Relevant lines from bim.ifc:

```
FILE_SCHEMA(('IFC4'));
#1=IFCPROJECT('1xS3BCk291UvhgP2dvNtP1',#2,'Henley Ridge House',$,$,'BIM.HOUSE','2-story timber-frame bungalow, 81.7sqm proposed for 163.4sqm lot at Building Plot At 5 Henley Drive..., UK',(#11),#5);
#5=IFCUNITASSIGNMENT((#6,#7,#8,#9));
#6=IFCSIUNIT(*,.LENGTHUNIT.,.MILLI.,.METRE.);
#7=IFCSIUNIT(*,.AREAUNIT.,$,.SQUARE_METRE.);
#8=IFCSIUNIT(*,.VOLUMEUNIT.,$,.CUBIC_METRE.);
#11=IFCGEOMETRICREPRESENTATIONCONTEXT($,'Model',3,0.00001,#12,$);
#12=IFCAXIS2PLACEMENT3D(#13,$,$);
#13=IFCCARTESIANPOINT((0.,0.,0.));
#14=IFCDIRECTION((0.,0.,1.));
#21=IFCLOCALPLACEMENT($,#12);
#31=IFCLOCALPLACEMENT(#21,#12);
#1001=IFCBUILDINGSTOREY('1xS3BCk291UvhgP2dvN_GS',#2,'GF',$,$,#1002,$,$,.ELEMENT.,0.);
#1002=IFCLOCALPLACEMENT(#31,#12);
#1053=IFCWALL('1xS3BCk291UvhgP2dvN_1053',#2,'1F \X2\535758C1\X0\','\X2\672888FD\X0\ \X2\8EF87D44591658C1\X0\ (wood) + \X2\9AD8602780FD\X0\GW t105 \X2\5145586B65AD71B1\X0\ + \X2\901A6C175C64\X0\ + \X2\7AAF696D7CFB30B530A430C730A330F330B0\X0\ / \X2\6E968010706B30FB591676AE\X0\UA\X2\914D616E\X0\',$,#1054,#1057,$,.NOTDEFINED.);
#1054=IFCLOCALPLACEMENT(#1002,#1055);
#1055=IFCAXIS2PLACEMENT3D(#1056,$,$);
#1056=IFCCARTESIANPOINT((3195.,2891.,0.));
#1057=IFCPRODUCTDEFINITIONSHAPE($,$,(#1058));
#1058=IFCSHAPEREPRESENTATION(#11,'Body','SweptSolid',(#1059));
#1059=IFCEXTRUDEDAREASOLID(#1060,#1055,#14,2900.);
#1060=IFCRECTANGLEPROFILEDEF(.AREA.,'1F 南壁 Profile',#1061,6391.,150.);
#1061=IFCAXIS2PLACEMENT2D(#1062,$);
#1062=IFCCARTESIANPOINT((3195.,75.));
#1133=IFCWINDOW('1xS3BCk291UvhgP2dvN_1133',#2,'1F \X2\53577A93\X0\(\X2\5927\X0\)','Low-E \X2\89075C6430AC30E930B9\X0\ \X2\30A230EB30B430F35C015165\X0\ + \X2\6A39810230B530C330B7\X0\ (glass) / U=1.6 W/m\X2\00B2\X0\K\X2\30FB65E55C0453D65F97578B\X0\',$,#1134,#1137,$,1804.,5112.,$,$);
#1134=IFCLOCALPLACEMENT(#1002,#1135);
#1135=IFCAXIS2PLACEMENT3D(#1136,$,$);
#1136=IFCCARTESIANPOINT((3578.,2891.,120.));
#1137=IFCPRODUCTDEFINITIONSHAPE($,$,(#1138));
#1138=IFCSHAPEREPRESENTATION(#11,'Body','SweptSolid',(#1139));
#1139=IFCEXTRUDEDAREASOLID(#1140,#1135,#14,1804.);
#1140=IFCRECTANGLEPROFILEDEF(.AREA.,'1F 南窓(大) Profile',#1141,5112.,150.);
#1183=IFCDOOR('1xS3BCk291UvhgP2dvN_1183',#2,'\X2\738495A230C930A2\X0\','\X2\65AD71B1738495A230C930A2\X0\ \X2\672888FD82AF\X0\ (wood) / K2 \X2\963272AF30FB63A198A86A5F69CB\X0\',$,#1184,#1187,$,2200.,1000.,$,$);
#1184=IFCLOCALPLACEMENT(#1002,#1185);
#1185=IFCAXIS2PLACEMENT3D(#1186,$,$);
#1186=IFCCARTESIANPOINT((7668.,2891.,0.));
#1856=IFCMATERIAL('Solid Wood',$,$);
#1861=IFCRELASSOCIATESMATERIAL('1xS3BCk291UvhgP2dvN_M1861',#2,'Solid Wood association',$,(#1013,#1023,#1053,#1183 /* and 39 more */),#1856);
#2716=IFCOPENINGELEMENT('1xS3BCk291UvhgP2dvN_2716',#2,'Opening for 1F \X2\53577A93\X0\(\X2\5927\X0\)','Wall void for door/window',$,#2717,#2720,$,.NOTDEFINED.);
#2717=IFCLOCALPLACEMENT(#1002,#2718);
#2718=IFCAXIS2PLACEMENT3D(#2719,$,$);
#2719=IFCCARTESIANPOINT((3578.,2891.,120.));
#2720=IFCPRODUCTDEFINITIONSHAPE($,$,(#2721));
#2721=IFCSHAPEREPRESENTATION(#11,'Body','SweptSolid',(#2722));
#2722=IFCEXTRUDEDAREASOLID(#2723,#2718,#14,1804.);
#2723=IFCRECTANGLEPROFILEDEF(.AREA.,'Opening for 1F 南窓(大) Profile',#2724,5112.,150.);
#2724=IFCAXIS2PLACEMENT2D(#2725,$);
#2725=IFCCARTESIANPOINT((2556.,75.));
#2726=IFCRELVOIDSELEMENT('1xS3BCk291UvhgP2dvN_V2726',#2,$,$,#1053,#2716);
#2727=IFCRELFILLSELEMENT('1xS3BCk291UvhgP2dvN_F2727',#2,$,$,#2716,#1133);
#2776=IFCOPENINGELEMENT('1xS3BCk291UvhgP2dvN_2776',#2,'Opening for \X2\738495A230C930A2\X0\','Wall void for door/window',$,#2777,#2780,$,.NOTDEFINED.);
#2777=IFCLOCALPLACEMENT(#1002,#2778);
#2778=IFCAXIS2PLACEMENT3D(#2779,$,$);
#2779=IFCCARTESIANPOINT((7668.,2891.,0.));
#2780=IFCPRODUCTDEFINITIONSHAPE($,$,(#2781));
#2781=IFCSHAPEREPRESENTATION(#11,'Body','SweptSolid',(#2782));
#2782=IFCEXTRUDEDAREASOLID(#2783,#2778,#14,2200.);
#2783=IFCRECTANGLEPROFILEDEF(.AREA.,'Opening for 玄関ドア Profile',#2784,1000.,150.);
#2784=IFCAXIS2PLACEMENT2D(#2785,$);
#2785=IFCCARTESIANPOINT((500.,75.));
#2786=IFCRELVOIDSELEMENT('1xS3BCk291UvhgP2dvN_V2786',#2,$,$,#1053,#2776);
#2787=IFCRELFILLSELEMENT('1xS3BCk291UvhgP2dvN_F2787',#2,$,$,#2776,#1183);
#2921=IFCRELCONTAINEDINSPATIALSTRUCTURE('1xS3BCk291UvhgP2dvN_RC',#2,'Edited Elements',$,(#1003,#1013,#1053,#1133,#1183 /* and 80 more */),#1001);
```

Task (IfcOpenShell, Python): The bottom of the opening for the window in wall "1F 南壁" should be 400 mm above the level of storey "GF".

```python
import numpy as np
import ifcopenshell
import ifcopenshell.api.geometry
import ifcopenshell.geom
import ifcopenshell.util.element
import ifcopenshell.util.placement
import ifcopenshell.util.shape
import ifcopenshell.util.unit

model = ifcopenshell.open("bim.ifc")
unit_scale = ifcopenshell.util.unit.calculate_unit_scale(model)

window = model.by_id(1133)
opening = window.FillsVoids[0].RelatingOpeningElement
storey = ifcopenshell.util.element.get_container(window, ifc_class="IfcBuildingStorey")
level = ifcopenshell.util.placement.get_local_placement(storey.ObjectPlacement)[2, 3]

# The opening's origin need not be at the sill, so measure its lowest point.
shape = ifcopenshell.geom.create_shape(ifcopenshell.geom.settings(), opening)
bottom = ifcopenshell.util.shape.get_shape_bottom_elevation(shape, shape.geometry) / unit_scale
dz = level + 0.4 / unit_scale - bottom

shift = np.array([0.0, 0.0, dz])
# The window is not placed relative to its opening, so move both.
for product in (opening, window):
    matrix = ifcopenshell.util.placement.get_local_placement(product.ObjectPlacement)
    matrix[:3, 3] += shift
    ifcopenshell.api.geometry.edit_object_placement(model, product=product, matrix=matrix, is_si=False)

print(f"moved by {dz * unit_scale:+.3f} m")

model.write("bim_updated.ifc")
```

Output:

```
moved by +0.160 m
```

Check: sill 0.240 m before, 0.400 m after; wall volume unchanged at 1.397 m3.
